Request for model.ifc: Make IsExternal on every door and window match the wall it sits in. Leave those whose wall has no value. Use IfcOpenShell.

First a look at what the model holds.

```python
import ifcopenshell
import ifcopenshell.util.element

model = ifcopenshell.open("model.ifc")
print(model.schema)
seen = {}
for e in model.by_type("IfcDoor") + model.by_type("IfcWindow"):
    if not e.FillsVoids:
        continue
    host = e.FillsVoids[0].RelatingOpeningElement.VoidsElements[0].RelatingBuildingElement
    own = ifcopenshell.util.element.get_pset(e, f"Pset_{e.is_a()[3:].removesuffix('StandardCase')}Common", "IsExternal")
    wall = ifcopenshell.util.element.get_pset(host, "Pset_WallCommon", "IsExternal")
    seen[e.is_a(), own, wall] = seen.get((e.is_a(), own, wall), 0) + 1
for (cls, own, wall), count in sorted(seen.items(), key=str):
    print(count, cls, "IsExternal:", own, "| host wall:", wall)
```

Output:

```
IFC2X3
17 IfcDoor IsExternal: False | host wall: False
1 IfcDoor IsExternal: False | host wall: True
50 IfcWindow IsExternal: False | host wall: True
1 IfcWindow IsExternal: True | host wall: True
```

```python
import ifcopenshell
import ifcopenshell.api.pset
import ifcopenshell.util.element

model = ifcopenshell.open("model.ifc")

count = 0
for ifc_class, pset_name in (("IfcDoor", "Pset_DoorCommon"), ("IfcWindow", "Pset_WindowCommon")):
    for e in model.by_type(ifc_class):
        if not e.FillsVoids:
            continue
        host = e.FillsVoids[0].RelatingOpeningElement.VoidsElements[0].RelatingBuildingElement
        external = ifcopenshell.util.element.get_pset(host, "Pset_WallCommon", "IsExternal")
        if external is None or ifcopenshell.util.element.get_pset(e, pset_name, "IsExternal") == external:
            continue
        pset = ifcopenshell.api.pset.add_pset(model, product=e, name=pset_name)
        ifcopenshell.api.pset.edit_pset(model, pset=pset, properties={"IsExternal": external})
        count += 1

print(count, "updated")

model.write("model_v2.ifc")
```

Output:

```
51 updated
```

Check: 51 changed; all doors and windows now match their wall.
